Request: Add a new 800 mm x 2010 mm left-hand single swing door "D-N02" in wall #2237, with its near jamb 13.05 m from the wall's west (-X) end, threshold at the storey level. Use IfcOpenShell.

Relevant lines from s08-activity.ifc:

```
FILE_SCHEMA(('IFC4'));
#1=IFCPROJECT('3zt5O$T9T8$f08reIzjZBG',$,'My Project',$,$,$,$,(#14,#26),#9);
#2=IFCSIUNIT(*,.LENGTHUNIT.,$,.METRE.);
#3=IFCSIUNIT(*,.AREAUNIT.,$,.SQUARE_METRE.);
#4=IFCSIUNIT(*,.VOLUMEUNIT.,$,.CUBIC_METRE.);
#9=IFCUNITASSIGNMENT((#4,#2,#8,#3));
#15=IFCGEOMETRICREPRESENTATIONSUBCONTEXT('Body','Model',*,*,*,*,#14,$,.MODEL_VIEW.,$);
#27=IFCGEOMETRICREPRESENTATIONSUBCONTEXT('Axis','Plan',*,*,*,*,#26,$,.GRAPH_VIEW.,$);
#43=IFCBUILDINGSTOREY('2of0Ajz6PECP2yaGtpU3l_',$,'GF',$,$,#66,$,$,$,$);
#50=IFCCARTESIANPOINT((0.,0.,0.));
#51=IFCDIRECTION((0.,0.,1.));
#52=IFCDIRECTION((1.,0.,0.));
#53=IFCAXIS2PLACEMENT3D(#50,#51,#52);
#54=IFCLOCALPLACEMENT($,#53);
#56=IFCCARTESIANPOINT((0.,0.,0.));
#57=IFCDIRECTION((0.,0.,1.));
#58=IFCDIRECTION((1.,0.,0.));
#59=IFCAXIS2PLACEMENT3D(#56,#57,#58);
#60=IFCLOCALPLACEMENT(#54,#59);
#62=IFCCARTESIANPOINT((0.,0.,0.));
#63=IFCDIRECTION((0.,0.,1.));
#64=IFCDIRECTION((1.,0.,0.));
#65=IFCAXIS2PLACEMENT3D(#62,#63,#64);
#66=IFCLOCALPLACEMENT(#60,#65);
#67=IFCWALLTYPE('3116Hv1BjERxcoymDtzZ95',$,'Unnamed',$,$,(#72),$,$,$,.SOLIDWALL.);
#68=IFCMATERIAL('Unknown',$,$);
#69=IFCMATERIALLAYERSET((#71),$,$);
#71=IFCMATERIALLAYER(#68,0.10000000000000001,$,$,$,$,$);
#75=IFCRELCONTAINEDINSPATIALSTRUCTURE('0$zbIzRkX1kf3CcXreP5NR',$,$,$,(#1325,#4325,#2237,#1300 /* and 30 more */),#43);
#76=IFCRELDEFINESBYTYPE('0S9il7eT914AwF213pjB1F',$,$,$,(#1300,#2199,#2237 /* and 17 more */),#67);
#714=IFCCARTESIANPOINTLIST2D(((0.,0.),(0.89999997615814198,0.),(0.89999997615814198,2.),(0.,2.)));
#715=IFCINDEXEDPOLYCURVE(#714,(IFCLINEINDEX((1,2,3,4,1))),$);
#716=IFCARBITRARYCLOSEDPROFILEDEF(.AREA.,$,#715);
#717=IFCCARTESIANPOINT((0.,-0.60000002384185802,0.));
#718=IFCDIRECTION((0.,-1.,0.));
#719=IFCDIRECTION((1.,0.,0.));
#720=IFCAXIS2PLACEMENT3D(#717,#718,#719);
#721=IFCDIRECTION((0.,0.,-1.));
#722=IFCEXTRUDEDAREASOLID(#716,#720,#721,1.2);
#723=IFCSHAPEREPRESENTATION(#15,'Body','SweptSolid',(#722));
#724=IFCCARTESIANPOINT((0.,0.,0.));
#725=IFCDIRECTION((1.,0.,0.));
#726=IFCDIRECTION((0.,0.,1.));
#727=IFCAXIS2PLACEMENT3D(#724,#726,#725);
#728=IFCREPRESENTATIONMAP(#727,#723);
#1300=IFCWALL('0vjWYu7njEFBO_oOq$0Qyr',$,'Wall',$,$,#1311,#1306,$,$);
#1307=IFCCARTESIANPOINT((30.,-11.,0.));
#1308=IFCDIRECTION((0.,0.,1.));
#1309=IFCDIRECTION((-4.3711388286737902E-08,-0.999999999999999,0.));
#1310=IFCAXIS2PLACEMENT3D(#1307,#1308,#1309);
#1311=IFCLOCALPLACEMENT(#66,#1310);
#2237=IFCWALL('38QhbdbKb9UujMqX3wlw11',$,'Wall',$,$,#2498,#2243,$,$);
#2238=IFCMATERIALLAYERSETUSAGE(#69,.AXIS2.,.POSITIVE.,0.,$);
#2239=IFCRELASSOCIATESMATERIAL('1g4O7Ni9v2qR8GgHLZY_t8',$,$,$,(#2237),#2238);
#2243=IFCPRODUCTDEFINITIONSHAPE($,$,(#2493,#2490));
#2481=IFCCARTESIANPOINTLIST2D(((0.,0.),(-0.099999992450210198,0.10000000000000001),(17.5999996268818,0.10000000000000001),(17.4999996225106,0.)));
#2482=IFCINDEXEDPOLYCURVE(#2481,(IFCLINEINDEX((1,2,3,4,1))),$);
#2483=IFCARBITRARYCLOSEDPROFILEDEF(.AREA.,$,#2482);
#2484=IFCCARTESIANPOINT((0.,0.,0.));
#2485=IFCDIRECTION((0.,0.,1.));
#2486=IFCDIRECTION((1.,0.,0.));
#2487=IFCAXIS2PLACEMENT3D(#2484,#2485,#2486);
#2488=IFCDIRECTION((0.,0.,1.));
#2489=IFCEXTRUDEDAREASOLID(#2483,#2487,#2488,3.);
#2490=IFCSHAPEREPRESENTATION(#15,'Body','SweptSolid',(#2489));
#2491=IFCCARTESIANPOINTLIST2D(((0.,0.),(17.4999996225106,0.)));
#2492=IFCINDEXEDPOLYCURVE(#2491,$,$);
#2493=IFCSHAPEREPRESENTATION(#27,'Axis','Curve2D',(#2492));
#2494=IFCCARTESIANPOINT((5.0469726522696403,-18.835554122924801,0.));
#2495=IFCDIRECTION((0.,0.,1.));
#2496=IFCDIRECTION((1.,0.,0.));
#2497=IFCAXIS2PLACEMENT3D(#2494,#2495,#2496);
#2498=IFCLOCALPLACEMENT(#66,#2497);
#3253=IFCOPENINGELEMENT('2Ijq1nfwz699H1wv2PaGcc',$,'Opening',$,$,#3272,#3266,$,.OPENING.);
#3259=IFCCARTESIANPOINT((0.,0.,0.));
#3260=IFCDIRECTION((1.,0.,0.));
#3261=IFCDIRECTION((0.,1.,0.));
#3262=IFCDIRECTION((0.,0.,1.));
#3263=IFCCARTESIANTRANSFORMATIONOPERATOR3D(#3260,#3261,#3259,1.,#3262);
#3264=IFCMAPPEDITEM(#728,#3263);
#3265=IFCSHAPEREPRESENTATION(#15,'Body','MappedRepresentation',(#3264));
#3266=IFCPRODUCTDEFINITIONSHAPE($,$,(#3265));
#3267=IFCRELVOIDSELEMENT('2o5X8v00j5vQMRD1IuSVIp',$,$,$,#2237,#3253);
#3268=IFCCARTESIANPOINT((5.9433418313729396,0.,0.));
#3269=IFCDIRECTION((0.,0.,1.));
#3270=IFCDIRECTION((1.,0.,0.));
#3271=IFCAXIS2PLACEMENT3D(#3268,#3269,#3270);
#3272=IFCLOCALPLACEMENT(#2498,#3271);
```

```python
import numpy as np
import ifcopenshell
import ifcopenshell.api.feature
import ifcopenshell.api.geometry
import ifcopenshell.api.root
import ifcopenshell.api.spatial
import ifcopenshell.geom
import ifcopenshell.util.element
import ifcopenshell.util.placement
import ifcopenshell.util.representation
import ifcopenshell.util.shape
import ifcopenshell.util.unit

model = ifcopenshell.open("s08-activity.ifc")
unit_scale = ifcopenshell.util.unit.calculate_unit_scale(model)
settings = ifcopenshell.geom.settings()


def volume(element):
    """Net volume in cubic metres, openings subtracted."""
    shape = ifcopenshell.geom.create_shape(settings, element)
    return ifcopenshell.util.shape.get_volume(shape.geometry)


wall = model.by_guid("38QhbdbKb9UujMqX3wlw11")
storey = ifcopenshell.util.element.get_container(wall, ifc_class="IfcBuildingStorey")
context = ifcopenshell.util.representation.get_context(model, "Model", "Body", "MODEL_VIEW")
before = volume(wall)

width, height, from_end, sill = 0.8, 2.01, 13.05, 0.0  # metres

# The wall runs along its own X axis, and the end named is its -X end.
wall_shape = ifcopenshell.geom.create_shape(settings, wall)
x, y, z = ifcopenshell.util.shape.get_vertices(wall_shape.geometry).T
start = x.min() + from_end
face, thickness = float(y.min()), float(y.max() - y.min())
wall_matrix = ifcopenshell.util.placement.get_local_placement(wall.ObjectPlacement)
level = ifcopenshell.util.placement.get_local_placement(storey.ObjectPlacement)[2, 3]


def in_wall(x, y):
    """Placement at x, y metres in the wall's axes, at sill height."""
    matrix = wall_matrix.copy()
    matrix[:, 3] = wall_matrix @ np.array([x / unit_scale, y / unit_scale, 0.0, 1.0])
    matrix[2, 3] = level + sill / unit_scale
    return matrix


# Opening: a box that overshoots both wall faces by 50 mm.
opening = ifcopenshell.api.root.create_entity(model, ifc_class="IfcOpeningElement", predefined_type="OPENING")
box = ifcopenshell.api.geometry.add_wall_representation(
    model, context=context, length=width, height=height, thickness=thickness + 0.1
)
ifcopenshell.api.geometry.assign_representation(model, product=opening, representation=box)
ifcopenshell.api.geometry.edit_object_placement(model, product=opening, matrix=in_wall(start, face - 0.05), is_si=False)
ifcopenshell.api.feature.add_feature(model, feature=opening, element=wall)

door = ifcopenshell.api.root.create_entity(model, ifc_class="IfcDoor", name="D-N02", predefined_type="DOOR")
door.OverallWidth, door.OverallHeight = width / unit_scale, height / unit_scale
door.OperationType = "SINGLE_SWING_LEFT"
body = ifcopenshell.api.geometry.add_door_representation(
    model,
    context=context,
    overall_width=door.OverallWidth,
    overall_height=door.OverallHeight,
    operation_type="SINGLE_SWING_LEFT",
    lining_properties={"LiningDepth": thickness / unit_scale, "ThresholdDepth": thickness / unit_scale},
)
ifcopenshell.api.geometry.assign_representation(model, product=door, representation=body)
ifcopenshell.api.spatial.assign_container(model, products=[door], relating_structure=storey)
ifcopenshell.api.feature.add_filling(model, opening=opening, element=door)

# The lining spans the wall, so the door starts at the wall face.
ifcopenshell.api.geometry.edit_object_placement(model, product=door, matrix=in_wall(start, face), is_si=False)

after = volume(wall)

print(f"wall volume {before:.3f} -> {after:.3f} m3")

model.write("s08-activity_edited.ifc")
```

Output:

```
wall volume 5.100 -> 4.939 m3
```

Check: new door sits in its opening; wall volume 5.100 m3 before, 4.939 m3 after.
